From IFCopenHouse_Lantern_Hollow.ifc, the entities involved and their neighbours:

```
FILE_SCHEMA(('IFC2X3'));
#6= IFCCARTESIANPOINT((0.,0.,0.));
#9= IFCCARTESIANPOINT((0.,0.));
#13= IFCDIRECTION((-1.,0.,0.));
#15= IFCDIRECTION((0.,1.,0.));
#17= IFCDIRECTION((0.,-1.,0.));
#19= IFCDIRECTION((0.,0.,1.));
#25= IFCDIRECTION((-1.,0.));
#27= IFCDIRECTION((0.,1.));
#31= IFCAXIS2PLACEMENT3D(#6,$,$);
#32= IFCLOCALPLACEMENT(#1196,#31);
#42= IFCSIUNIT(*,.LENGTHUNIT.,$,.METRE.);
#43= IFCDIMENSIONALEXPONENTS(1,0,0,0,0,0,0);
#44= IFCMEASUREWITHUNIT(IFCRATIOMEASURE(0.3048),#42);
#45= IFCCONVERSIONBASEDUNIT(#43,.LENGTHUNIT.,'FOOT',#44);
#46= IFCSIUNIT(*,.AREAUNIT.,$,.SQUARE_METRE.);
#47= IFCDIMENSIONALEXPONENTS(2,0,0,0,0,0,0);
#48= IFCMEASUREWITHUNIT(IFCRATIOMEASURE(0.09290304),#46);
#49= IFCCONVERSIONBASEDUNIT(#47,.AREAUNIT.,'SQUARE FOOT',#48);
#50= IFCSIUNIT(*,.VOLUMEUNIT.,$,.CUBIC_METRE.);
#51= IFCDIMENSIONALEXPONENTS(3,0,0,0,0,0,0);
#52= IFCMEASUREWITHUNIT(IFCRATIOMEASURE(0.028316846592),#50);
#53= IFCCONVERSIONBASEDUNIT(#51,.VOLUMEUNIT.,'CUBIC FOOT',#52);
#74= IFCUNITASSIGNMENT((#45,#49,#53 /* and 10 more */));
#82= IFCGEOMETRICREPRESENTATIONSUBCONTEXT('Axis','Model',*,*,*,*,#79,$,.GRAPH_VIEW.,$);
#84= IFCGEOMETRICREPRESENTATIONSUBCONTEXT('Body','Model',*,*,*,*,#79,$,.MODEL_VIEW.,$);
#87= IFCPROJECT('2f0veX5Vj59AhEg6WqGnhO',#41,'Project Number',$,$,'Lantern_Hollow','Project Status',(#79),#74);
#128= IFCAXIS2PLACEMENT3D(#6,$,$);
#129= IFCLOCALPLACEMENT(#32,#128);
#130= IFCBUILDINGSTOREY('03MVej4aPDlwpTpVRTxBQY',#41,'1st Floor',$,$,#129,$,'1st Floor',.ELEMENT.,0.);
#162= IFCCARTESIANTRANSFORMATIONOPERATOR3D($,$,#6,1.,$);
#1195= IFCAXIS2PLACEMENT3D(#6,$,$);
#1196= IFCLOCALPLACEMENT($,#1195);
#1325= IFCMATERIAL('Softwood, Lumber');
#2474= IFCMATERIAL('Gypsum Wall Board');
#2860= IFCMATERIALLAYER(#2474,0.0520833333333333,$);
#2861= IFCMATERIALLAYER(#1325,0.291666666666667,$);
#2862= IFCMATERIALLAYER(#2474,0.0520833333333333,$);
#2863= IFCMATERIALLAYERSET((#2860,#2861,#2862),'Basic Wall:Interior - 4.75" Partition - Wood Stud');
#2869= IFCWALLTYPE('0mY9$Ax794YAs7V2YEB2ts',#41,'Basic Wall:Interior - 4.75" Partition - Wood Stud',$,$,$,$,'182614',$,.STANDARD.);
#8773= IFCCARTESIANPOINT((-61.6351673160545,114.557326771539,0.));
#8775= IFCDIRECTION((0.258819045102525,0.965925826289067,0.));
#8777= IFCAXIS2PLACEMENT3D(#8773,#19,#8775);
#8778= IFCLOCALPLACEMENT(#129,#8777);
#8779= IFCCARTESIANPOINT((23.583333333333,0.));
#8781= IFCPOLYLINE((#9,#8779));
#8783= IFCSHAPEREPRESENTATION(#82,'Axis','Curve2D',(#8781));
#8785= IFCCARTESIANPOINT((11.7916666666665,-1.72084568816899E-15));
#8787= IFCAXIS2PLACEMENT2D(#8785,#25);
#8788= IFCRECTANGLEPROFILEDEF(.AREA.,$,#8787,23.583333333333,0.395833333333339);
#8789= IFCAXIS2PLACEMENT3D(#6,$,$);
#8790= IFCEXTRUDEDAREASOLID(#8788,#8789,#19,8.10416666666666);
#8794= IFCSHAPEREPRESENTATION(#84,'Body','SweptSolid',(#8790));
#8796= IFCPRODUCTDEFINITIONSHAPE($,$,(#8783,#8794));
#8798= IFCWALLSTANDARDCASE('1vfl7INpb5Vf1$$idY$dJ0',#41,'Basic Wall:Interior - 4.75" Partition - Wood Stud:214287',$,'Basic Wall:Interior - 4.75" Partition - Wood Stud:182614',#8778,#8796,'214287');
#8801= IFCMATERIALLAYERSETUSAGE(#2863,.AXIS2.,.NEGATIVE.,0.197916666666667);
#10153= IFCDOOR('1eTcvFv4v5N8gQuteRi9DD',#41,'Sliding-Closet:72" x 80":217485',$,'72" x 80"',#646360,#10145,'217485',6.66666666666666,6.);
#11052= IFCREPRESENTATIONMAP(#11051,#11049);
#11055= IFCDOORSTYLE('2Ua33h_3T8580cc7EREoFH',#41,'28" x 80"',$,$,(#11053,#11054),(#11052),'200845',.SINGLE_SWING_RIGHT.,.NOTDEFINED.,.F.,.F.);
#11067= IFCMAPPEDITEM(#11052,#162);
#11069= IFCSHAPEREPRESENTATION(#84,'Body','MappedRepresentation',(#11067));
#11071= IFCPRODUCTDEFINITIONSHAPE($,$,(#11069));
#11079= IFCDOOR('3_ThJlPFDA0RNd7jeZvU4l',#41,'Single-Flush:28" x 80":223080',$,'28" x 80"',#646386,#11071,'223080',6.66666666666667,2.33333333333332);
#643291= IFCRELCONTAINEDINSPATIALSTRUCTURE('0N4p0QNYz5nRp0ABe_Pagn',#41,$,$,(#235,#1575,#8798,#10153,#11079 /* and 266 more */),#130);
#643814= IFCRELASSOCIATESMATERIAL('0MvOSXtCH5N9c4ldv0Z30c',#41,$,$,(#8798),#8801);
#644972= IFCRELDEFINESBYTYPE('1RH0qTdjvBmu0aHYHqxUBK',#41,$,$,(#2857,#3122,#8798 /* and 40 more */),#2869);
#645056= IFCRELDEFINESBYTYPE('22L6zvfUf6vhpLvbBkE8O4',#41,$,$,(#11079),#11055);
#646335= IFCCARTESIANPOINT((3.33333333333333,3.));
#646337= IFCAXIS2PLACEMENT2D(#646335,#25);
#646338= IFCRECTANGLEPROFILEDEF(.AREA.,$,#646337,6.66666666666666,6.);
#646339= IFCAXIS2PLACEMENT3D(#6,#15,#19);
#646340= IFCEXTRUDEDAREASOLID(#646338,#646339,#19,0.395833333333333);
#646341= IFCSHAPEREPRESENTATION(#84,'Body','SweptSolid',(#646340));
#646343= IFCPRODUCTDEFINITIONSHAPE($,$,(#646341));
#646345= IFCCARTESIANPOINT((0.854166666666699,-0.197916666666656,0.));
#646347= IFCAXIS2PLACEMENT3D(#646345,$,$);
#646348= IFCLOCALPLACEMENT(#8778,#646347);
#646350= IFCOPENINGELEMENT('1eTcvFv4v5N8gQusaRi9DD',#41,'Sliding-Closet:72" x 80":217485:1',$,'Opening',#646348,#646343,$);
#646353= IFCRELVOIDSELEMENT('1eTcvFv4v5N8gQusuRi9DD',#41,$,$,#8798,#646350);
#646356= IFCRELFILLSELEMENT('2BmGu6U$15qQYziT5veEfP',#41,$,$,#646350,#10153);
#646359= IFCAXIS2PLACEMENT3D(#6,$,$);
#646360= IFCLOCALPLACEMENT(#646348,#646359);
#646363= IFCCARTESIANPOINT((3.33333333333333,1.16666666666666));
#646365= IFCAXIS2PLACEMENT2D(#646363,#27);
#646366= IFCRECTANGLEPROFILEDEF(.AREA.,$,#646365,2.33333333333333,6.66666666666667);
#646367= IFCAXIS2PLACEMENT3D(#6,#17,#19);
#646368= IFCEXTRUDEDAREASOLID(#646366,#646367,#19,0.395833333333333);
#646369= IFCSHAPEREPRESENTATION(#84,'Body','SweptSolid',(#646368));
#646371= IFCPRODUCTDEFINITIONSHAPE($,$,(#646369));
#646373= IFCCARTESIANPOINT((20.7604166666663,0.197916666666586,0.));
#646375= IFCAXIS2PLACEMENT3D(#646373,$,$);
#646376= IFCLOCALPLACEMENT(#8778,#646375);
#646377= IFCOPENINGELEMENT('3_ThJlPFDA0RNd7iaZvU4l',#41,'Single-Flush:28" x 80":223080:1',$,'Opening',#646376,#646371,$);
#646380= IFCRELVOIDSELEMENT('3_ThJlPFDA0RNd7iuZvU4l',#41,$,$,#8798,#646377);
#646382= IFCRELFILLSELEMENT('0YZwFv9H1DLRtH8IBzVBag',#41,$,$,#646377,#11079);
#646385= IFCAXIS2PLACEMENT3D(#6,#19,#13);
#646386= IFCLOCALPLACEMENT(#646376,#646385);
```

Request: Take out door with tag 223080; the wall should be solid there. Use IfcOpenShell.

```python
import ifcopenshell
import ifcopenshell.api.feature
import ifcopenshell.api.root
import ifcopenshell.geom
import ifcopenshell.util.shape

model = ifcopenshell.open("IFCopenHouse_Lantern_Hollow.ifc")
settings = ifcopenshell.geom.settings()


def volume(element):
    """Net volume in cubic metres, openings subtracted."""
    shape = ifcopenshell.geom.create_shape(settings, element)
    return ifcopenshell.util.shape.get_volume(shape.geometry)


door = model.by_guid("3_ThJlPFDA0RNd7jeZvU4l")
opening = door.FillsVoids[0].RelatingOpeningElement
wall = opening.VoidsElements[0].RelatingBuildingElement
before = volume(wall)

ifcopenshell.api.root.remove_product(model, product=door)
ifcopenshell.api.feature.remove_feature(model, feature=opening)

after = volume(wall)

print(f"wall volume {before:.3f} -> {after:.3f} m3")

model.write("IFCopenHouse_Lantern_Hollow_edited.ifc")
```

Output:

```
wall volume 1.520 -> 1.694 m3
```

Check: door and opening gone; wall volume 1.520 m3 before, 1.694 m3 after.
